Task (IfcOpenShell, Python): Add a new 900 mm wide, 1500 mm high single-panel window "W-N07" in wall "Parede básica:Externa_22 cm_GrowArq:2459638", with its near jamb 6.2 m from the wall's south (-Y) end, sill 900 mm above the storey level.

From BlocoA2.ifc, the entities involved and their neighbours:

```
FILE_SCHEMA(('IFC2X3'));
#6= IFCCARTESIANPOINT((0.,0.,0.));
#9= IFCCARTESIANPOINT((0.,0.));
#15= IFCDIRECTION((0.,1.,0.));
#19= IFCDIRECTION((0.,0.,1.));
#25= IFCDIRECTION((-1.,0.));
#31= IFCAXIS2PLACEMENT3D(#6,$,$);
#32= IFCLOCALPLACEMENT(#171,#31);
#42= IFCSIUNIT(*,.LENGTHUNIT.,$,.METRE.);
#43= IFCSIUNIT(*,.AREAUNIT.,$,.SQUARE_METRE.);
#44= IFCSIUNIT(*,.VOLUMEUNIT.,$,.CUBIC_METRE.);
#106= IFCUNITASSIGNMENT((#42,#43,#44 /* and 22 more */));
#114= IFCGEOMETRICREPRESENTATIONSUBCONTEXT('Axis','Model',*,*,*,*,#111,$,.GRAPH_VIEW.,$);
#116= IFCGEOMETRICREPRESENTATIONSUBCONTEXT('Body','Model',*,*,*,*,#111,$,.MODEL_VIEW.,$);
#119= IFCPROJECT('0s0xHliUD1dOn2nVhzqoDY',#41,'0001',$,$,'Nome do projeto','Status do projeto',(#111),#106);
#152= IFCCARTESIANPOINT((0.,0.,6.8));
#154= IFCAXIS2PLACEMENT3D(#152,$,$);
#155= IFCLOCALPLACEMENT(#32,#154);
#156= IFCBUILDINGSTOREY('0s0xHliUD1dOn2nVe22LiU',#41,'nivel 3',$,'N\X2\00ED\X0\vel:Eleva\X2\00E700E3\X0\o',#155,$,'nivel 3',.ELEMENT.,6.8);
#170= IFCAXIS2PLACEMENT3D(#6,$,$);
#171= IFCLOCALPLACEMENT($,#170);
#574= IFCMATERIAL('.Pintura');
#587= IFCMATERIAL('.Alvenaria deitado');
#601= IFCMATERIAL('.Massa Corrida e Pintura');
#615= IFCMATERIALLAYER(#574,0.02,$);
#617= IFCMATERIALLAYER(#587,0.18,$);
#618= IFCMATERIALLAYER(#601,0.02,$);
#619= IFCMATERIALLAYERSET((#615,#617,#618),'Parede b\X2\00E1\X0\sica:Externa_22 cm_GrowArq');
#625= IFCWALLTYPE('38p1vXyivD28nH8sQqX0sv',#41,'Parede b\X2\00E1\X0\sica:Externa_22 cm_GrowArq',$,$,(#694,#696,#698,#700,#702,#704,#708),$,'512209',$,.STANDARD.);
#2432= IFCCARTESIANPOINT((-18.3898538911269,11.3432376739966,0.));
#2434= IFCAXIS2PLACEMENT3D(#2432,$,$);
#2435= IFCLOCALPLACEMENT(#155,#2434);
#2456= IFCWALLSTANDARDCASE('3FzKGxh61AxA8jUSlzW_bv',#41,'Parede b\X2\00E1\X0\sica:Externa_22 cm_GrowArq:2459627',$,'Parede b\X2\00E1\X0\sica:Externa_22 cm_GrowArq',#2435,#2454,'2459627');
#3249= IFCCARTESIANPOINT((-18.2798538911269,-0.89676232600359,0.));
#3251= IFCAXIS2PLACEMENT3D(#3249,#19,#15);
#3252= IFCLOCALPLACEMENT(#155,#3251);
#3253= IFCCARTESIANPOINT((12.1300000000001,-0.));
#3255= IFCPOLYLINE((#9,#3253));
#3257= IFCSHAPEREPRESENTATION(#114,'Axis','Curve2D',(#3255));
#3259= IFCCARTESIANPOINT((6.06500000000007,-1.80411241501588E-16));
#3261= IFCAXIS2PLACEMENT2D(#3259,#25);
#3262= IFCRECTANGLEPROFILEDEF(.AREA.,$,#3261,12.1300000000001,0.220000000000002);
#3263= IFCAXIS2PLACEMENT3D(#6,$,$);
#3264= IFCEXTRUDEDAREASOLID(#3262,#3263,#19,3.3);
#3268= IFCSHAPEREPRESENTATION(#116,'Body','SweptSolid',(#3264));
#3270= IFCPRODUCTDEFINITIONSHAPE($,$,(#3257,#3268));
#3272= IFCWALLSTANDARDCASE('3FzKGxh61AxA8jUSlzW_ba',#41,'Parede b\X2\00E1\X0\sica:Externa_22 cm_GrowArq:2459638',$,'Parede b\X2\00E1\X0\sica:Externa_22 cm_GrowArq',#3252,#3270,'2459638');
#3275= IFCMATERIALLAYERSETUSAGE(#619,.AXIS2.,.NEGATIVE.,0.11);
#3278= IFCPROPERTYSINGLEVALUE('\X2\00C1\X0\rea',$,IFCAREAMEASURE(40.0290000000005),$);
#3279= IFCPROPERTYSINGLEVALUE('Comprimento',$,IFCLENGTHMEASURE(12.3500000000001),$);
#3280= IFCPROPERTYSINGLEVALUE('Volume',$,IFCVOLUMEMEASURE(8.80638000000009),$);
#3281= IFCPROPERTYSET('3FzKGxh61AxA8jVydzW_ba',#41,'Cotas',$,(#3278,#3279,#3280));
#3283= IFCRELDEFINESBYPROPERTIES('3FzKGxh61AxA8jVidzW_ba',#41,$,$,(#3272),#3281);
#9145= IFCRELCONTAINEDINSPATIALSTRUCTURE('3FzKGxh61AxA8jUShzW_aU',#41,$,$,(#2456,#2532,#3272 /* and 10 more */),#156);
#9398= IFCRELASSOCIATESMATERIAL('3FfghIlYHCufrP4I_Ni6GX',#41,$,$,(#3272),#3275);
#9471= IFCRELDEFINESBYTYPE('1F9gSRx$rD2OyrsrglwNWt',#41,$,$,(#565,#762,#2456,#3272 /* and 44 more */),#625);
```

```python
import numpy as np
import ifcopenshell
import ifcopenshell.api.feature
import ifcopenshell.api.geometry
import ifcopenshell.api.pset
import ifcopenshell.api.root
import ifcopenshell.api.spatial
import ifcopenshell.api.type
import ifcopenshell.geom
import ifcopenshell.util.element
import ifcopenshell.util.placement
import ifcopenshell.util.representation
import ifcopenshell.util.shape
import ifcopenshell.util.unit

model = ifcopenshell.open("BlocoA2.ifc")
unit_scale = ifcopenshell.util.unit.calculate_unit_scale(model)
area_scale = ifcopenshell.util.unit.calculate_unit_scale(model, "AREAUNIT")
volume_scale = ifcopenshell.util.unit.calculate_unit_scale(model, "VOLUMEUNIT")
settings = ifcopenshell.geom.settings()


def volume(element):
    """Net volume in cubic metres, openings subtracted."""
    shape = ifcopenshell.geom.create_shape(settings, element)
    return ifcopenshell.util.shape.get_volume(shape.geometry)


wall = model.by_guid("3FzKGxh61AxA8jUSlzW_ba")
storey = ifcopenshell.util.element.get_container(wall, ifc_class="IfcBuildingStorey")
context = ifcopenshell.util.representation.get_context(model, "Model", "Body", "MODEL_VIEW")
before = volume(wall)

width, height, from_end, sill = 0.9, 1.5, 6.2, 0.9  # metres

# The wall runs along its own X axis, and the end named is its -X end.
wall_shape = ifcopenshell.geom.create_shape(settings, wall)
x, y, z = ifcopenshell.util.shape.get_vertices(wall_shape.geometry).T
start = x.min() + from_end
face, thickness = float(y.min()), float(y.max() - y.min())
wall_matrix = ifcopenshell.util.placement.get_local_placement(wall.ObjectPlacement)
level = ifcopenshell.util.placement.get_local_placement(storey.ObjectPlacement)[2, 3]


def in_wall(x, y):
    """Placement at x, y metres in the wall's axes, at sill height."""
    matrix = wall_matrix.copy()
    matrix[:, 3] = wall_matrix @ np.array([x / unit_scale, y / unit_scale, 0.0, 1.0])
    matrix[2, 3] = level + sill / unit_scale
    return matrix


# Opening: a box that overshoots both wall faces by 50 mm.
opening = ifcopenshell.api.root.create_entity(model, ifc_class="IfcOpeningElement")
box = ifcopenshell.api.geometry.add_wall_representation(
    model, context=context, length=width, height=height, thickness=thickness + 0.1
)
ifcopenshell.api.geometry.assign_representation(model, product=opening, representation=box)
ifcopenshell.api.geometry.edit_object_placement(model, product=opening, matrix=in_wall(start, face - 0.05), is_si=False)
ifcopenshell.api.feature.add_feature(model, feature=opening, element=wall)

window = ifcopenshell.api.root.create_entity(model, ifc_class="IfcWindow", name="W-N07")
window.OverallWidth, window.OverallHeight = width / unit_scale, height / unit_scale
body = ifcopenshell.api.geometry.add_window_representation(
    model,
    context=context,
    overall_width=window.OverallWidth,
    overall_height=window.OverallHeight,
    partition_type="SINGLE_PANEL",
)
ifcopenshell.api.geometry.assign_representation(model, product=window, representation=body)
ifcopenshell.api.spatial.assign_container(model, products=[window], relating_structure=storey)
fills = ifcopenshell.api.feature.add_filling(model, opening=opening, element=window)
fills.OwnerHistory = window.OwnerHistory  # required in IFC2X3

# IFC2X3 keeps the operation on the window style.
style = ifcopenshell.api.root.create_entity(model, ifc_class="IfcWindowStyle", name="W-N07")
style.OperationType, style.ConstructionType = "SINGLE_PANEL", "NOTDEFINED"
style.ParameterTakesPrecedence = style.Sizeable = False
ifcopenshell.api.type.assign_type(model, related_objects=[window], relating_type=style)

# Centre the window in the wall's thickness.
ifcopenshell.api.geometry.edit_object_placement(model, product=window, matrix=in_wall(start, face), is_si=False)
window_shape = ifcopenshell.geom.create_shape(settings, window)
depth = ifcopenshell.util.shape.get_vertices(window_shape.geometry)[:, 1]
offset = face + thickness / 2 - (depth.min() + depth.max()) / 2
ifcopenshell.api.geometry.edit_object_placement(model, product=window, matrix=in_wall(start, offset), is_si=False)

after = volume(wall)

# Update the wall's stored quantities.
pset = model.by_id(ifcopenshell.util.element.get_pset(wall, "Cotas", should_inherit=False)["id"])
ifcopenshell.api.pset.edit_pset(model, pset=pset, properties={
    "Área": model.create_entity("IfcAreaMeasure", after / thickness / area_scale),
    "Volume": model.create_entity("IfcVolumeMeasure", after / volume_scale),
})

print(f"wall volume {before:.3f} -> {after:.3f} m3")

model.write("BlocoA2_rev.ifc")
```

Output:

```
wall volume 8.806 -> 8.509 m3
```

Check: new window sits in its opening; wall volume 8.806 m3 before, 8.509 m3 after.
